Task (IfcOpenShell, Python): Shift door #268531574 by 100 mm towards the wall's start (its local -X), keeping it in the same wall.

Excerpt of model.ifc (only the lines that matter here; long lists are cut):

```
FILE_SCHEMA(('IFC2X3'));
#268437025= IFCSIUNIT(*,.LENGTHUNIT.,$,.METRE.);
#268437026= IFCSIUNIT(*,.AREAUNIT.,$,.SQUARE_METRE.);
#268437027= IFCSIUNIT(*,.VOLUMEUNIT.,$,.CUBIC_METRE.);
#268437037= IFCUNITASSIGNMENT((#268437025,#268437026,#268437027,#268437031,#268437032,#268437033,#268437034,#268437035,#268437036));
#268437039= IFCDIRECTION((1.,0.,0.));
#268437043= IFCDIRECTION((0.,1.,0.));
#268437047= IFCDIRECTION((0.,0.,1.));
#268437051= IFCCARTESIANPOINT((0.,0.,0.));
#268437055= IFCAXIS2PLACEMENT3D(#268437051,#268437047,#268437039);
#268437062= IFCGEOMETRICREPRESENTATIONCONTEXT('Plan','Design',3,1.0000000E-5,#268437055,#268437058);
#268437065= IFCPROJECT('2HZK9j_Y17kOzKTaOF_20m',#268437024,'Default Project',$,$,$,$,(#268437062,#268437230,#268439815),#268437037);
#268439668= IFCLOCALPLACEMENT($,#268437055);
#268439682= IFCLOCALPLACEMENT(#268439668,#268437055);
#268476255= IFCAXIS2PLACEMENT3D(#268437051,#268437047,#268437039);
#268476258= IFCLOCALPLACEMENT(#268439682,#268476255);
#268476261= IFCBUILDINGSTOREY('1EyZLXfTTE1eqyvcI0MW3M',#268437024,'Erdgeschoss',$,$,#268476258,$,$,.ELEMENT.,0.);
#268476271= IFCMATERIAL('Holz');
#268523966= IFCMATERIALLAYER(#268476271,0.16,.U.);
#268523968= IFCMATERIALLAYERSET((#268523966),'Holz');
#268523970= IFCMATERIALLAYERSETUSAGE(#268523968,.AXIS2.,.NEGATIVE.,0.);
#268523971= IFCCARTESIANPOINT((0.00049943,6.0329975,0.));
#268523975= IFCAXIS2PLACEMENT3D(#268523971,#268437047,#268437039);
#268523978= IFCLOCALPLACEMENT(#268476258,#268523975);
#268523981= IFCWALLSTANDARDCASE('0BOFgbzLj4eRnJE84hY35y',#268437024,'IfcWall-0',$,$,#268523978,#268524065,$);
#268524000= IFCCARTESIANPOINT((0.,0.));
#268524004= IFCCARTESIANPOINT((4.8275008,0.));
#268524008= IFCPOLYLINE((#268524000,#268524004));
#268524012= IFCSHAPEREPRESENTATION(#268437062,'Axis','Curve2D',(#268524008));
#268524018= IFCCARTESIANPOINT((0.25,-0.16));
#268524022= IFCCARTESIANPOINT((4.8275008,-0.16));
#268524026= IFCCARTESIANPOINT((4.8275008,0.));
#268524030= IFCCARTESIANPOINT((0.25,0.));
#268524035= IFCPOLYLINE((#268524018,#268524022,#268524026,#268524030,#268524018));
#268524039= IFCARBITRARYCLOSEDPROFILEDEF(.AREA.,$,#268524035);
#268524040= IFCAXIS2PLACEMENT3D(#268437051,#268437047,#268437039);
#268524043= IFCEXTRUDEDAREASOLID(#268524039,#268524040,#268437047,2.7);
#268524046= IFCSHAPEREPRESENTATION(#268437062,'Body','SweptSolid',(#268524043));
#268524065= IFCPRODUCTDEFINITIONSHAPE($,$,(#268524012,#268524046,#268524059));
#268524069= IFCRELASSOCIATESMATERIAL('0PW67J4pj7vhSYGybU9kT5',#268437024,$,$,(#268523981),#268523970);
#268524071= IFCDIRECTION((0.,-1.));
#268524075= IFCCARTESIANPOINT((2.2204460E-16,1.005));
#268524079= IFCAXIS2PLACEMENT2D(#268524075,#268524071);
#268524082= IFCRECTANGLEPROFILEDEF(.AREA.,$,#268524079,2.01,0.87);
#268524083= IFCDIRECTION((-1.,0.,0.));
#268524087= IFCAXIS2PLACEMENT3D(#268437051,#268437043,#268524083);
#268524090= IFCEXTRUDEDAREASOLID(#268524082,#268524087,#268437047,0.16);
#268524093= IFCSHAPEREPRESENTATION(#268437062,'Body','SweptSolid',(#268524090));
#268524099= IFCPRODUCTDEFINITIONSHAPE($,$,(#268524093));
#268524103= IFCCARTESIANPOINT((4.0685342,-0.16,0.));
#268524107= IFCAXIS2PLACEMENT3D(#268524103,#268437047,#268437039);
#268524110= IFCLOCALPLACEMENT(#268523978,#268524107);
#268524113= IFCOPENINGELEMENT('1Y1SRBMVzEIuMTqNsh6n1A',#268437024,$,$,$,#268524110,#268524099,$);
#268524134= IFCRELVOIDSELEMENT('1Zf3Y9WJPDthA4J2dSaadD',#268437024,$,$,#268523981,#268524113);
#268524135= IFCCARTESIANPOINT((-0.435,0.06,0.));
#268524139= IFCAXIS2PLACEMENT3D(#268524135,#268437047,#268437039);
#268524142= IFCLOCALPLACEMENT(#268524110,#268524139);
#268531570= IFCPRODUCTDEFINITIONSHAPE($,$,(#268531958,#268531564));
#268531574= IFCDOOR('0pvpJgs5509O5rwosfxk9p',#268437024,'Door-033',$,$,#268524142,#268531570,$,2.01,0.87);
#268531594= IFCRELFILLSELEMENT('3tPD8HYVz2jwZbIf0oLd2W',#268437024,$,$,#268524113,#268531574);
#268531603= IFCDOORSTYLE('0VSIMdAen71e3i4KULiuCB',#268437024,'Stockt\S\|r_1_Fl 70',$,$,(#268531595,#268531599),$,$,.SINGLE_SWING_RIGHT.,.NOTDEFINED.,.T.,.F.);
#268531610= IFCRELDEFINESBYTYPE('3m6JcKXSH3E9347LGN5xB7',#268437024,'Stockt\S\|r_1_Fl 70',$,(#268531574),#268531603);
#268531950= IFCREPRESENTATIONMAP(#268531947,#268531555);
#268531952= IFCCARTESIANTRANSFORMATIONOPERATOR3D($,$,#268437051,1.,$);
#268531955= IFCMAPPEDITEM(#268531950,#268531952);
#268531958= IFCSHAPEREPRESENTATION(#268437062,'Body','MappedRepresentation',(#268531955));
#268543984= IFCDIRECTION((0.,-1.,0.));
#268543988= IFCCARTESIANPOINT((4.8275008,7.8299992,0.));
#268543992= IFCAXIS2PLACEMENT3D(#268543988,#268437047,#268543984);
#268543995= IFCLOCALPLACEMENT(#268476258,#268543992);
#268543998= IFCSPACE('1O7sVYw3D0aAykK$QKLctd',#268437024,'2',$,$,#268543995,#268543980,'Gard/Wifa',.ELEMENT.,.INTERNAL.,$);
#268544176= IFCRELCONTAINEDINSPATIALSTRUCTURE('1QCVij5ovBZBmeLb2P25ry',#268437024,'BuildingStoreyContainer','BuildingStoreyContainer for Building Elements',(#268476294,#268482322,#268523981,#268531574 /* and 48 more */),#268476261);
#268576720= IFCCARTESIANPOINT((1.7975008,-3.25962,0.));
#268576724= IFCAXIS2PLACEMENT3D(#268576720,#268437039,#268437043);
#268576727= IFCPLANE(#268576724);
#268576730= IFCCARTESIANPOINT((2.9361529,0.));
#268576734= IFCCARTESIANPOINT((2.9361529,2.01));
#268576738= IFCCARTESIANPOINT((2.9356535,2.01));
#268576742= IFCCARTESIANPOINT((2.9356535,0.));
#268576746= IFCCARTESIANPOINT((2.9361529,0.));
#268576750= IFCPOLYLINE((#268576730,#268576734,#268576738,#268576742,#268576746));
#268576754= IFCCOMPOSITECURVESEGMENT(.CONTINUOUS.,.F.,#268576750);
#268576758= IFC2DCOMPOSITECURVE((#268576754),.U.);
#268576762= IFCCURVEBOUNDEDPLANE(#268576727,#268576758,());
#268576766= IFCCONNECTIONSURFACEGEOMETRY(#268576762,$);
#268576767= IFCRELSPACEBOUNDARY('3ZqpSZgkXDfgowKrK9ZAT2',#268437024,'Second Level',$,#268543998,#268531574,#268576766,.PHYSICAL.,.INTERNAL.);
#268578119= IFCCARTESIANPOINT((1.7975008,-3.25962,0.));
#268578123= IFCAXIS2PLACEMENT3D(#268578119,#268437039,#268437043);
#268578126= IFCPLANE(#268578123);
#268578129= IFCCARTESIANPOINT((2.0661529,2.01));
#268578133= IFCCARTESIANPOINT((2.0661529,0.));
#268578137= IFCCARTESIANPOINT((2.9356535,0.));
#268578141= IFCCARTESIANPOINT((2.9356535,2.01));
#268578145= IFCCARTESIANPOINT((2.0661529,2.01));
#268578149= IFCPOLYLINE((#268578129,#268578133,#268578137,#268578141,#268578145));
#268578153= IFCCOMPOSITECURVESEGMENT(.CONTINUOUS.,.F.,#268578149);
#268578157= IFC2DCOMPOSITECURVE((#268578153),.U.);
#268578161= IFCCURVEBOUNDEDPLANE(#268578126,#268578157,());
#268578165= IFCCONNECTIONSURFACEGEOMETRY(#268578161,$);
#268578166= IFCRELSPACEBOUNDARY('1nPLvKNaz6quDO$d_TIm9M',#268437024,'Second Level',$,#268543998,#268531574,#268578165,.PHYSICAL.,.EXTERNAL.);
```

```python
import numpy as np
import ifcopenshell
import ifcopenshell.api.geometry
import ifcopenshell.util.placement
import ifcopenshell.util.unit

model = ifcopenshell.open("model.ifc")
unit_scale = ifcopenshell.util.unit.calculate_unit_scale(model)

door = model.by_id(268531574)
opening = door.FillsVoids[0].RelatingOpeningElement
wall = opening.VoidsElements[0].RelatingBuildingElement

wall_matrix = ifcopenshell.util.placement.get_local_placement(wall.ObjectPlacement)
shift = wall_matrix[:3, 0] * -0.1 / unit_scale
before = ifcopenshell.util.placement.get_local_placement(door.ObjectPlacement)[:3, 3].copy()

# The door is placed relative to its opening, so it follows when the opening moves.
matrix = ifcopenshell.util.placement.get_local_placement(opening.ObjectPlacement)
matrix[:3, 3] += shift
ifcopenshell.api.geometry.edit_object_placement(
    model, product=opening, matrix=matrix, is_si=False, should_transform_children=True
)

# Space boundary surfaces are stored in each space's coordinates; move them too.
for rel in door.ProvidesBoundaries:
    if not rel.ConnectionGeometry:
        continue
    surface = rel.ConnectionGeometry.SurfaceOnRelatingElement.BasisSurface
    space_matrix = ifcopenshell.util.placement.get_local_placement(rel.RelatingSpace.ObjectPlacement)
    point = np.array(surface.Position.Location.Coordinates) + space_matrix[:3, :3].T @ shift
    surface.Position = model.createIfcAxis2Placement3D(
        model.createIfcCartesianPoint(point.tolist()), surface.Position.Axis, surface.Position.RefDirection
    )

after = ifcopenshell.util.placement.get_local_placement(door.ObjectPlacement)[:3, 3]
print("door moved by", (after - before).round(3) + 0.0)

model.write("model-out.ifc")
```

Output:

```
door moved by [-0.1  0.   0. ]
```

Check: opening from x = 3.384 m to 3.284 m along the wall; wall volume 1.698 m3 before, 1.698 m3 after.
